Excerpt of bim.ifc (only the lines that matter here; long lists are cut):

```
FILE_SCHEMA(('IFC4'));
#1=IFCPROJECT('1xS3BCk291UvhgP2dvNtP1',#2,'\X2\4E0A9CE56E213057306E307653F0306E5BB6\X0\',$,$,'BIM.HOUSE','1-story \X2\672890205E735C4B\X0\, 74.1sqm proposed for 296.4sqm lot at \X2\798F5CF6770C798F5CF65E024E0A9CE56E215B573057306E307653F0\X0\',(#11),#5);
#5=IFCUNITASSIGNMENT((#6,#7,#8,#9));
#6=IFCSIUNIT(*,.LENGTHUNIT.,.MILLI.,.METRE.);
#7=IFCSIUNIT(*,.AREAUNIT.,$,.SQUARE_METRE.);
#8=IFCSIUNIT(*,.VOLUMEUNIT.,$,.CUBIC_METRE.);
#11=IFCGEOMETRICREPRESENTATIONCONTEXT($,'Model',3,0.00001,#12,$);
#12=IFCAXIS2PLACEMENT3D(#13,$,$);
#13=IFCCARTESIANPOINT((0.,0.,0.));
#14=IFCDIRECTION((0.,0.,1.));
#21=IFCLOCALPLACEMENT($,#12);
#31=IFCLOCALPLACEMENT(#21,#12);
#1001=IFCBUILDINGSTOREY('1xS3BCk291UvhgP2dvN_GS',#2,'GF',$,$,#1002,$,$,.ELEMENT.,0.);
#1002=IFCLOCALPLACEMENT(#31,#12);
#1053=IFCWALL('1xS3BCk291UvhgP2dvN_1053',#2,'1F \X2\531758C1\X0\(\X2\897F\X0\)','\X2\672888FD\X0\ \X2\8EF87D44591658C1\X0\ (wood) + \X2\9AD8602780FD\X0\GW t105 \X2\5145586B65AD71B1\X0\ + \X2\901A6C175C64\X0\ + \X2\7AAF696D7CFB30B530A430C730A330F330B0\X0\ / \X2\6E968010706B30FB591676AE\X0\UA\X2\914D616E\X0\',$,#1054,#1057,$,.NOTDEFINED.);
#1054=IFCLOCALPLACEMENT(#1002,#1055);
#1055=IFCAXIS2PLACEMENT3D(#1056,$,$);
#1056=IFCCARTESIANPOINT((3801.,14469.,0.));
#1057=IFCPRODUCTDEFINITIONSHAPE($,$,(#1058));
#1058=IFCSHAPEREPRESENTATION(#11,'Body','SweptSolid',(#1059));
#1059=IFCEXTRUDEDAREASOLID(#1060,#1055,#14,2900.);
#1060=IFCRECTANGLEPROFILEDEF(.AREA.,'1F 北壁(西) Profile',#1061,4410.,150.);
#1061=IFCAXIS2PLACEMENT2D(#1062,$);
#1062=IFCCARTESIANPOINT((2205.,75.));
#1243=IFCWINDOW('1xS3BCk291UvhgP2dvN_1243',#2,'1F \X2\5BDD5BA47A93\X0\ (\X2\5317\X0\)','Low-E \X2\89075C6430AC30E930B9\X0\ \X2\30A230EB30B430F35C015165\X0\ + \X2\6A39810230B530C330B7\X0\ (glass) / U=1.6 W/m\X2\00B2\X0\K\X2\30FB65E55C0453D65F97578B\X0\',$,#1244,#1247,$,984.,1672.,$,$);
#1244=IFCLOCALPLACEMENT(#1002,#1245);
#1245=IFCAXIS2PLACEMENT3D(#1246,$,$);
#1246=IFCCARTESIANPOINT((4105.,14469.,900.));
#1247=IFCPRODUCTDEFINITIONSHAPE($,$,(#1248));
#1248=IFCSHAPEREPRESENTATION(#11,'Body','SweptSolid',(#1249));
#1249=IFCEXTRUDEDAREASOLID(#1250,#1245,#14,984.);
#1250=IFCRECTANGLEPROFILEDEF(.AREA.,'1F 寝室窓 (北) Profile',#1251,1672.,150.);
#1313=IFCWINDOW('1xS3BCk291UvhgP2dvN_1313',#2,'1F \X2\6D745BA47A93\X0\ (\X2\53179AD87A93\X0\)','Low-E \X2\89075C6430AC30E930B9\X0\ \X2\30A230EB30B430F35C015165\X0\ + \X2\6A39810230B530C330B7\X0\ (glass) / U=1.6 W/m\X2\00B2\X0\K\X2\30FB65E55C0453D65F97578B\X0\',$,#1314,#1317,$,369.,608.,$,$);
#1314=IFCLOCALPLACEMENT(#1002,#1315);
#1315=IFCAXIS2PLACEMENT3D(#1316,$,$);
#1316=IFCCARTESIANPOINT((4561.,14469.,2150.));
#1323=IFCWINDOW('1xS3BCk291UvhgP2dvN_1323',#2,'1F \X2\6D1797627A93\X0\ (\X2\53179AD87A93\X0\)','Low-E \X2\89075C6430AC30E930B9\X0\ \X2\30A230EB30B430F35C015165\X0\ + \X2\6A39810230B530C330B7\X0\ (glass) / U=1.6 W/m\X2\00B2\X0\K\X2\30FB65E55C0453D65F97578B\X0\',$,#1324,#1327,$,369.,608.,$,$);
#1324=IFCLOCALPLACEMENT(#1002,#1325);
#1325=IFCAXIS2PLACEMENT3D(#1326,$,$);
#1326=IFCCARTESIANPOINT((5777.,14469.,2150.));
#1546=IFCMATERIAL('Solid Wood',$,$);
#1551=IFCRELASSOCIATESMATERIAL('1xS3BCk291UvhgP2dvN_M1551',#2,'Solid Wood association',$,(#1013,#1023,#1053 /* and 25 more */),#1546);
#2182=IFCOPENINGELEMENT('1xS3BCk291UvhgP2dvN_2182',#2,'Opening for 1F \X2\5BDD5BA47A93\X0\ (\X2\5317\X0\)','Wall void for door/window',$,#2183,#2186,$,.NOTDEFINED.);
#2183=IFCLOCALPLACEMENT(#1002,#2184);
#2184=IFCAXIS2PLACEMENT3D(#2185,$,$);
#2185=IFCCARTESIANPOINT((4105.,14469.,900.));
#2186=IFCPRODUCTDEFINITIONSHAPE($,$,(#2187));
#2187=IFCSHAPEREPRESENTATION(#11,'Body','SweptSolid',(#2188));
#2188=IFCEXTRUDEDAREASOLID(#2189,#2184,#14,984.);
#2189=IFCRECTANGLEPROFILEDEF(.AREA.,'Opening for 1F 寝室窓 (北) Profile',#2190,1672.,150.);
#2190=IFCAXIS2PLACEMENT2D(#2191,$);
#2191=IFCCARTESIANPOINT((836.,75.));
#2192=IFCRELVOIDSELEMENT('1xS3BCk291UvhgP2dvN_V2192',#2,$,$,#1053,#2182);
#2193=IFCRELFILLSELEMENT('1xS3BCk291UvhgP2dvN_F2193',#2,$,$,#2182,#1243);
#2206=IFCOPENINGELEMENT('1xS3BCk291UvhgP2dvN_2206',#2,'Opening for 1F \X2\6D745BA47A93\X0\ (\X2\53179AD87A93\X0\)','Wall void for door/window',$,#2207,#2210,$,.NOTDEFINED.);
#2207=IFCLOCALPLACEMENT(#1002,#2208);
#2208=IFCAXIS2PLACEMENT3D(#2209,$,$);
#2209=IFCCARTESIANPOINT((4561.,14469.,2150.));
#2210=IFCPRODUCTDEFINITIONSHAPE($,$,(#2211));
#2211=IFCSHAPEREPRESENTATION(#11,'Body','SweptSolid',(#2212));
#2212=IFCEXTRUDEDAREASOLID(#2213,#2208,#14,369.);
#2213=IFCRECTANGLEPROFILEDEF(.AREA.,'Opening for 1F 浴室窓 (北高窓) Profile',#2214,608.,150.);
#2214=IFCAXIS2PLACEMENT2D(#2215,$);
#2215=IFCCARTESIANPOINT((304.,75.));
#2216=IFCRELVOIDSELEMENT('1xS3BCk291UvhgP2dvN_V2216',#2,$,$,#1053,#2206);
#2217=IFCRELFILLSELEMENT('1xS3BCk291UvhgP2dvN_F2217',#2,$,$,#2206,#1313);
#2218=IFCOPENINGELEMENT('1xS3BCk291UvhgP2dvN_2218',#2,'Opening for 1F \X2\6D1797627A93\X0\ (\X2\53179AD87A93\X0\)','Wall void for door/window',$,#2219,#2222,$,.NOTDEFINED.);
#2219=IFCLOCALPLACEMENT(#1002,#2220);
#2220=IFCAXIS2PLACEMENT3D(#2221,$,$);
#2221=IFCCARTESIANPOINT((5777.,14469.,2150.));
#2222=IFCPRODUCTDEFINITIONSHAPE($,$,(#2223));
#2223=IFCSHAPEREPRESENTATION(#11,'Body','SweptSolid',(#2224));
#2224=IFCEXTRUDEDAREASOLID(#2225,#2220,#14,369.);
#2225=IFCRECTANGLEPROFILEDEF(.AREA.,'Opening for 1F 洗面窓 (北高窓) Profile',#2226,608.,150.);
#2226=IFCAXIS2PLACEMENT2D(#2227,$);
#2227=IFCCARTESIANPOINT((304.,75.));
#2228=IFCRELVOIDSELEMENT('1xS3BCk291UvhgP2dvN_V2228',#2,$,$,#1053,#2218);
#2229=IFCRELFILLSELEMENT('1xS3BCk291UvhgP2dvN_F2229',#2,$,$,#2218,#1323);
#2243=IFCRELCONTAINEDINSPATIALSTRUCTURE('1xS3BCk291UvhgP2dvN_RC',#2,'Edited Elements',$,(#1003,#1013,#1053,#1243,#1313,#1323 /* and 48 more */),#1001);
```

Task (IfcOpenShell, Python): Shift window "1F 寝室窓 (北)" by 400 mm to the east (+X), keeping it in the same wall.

```python
import ifcopenshell
import ifcopenshell.api.geometry
import ifcopenshell.util.placement

model = ifcopenshell.open("bim.ifc")

window = model.by_guid("1xS3BCk291UvhgP2dvN_1243")
opening = window.FillsVoids[0].RelatingOpeningElement
wall = opening.VoidsElements[0].RelatingBuildingElement

wall_matrix = ifcopenshell.util.placement.get_local_placement(wall.ObjectPlacement)
shift = wall_matrix[:3, 0] * 400.0
before = ifcopenshell.util.placement.get_local_placement(window.ObjectPlacement)[:3, 3].copy()

# The window is not placed relative to its opening, so move both.
for product in (opening, window):
    matrix = ifcopenshell.util.placement.get_local_placement(product.ObjectPlacement)
    matrix[:3, 3] += shift
    ifcopenshell.api.geometry.edit_object_placement(model, product=product, matrix=matrix, is_si=False)

after = ifcopenshell.util.placement.get_local_placement(window.ObjectPlacement)[:3, 3]
print("window moved by", (after - before).round(3) + 0.0)

model.write("bim_edited.ifc")
```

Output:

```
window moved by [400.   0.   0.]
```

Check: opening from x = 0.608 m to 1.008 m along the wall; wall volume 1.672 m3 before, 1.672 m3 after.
